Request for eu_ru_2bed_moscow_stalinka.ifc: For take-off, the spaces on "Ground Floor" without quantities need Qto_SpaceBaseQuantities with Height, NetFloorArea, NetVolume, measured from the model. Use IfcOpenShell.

First a look at what the model holds.

```python
import ifcopenshell
import ifcopenshell.util.element
import ifcopenshell.util.unit

model = ifcopenshell.open("eu_ru_2bed_moscow_stalinka.ifc")
print(model.schema)
for unit_type in ("LENGTHUNIT", "AREAUNIT", "VOLUMEUNIT"):
    print(unit_type, ifcopenshell.util.unit.calculate_unit_scale(model, unit_type))
storey = next(s for s in model.by_type("IfcBuildingStorey") if s.Name == "Ground Floor")
spaces = [e for e in ifcopenshell.util.element.get_decomposition(storey) if e.is_a("IfcSpace")]
for e in sorted(spaces, key=lambda e: e.id()):
    print(e.id(), e.is_a(), e.Name, list(ifcopenshell.util.element.get_psets(e, qtos_only=True)), sep=" | ")
```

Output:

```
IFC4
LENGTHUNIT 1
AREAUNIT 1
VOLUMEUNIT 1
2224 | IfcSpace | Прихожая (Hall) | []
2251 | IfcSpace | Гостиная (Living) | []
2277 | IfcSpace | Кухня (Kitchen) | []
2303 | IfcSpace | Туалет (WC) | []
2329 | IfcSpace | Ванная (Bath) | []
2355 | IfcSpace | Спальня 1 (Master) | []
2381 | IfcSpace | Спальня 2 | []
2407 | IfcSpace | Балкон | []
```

```python
import ifcopenshell
import ifcopenshell.api.pset
import ifcopenshell.geom
import ifcopenshell.util.element
import ifcopenshell.util.shape
import ifcopenshell.util.unit

model = ifcopenshell.open("eu_ru_2bed_moscow_stalinka.ifc")
unit_scale = ifcopenshell.util.unit.calculate_unit_scale(model)
area_scale = ifcopenshell.util.unit.calculate_unit_scale(model, "AREAUNIT")
volume_scale = ifcopenshell.util.unit.calculate_unit_scale(model, "VOLUMEUNIT")
settings = ifcopenshell.geom.settings()

storey = next(s for s in model.by_type("IfcBuildingStorey") if s.Name == "Ground Floor")
spaces = [e for e in ifcopenshell.util.element.get_decomposition(storey) if e.is_a("IfcSpace")]

for e in sorted(spaces, key=lambda e: e.id()):
    if ifcopenshell.util.element.get_psets(e, qtos_only=True, should_inherit=False):
        continue
    # Geometry comes back in metres, in the element's own axes.
    shape = ifcopenshell.geom.create_shape(settings, e)
    values = {
        "Height": ifcopenshell.util.shape.get_z(shape.geometry) / unit_scale,
        "NetFloorArea": ifcopenshell.util.shape.get_footprint_area(shape.geometry) / area_scale,
        "NetVolume": ifcopenshell.util.shape.get_volume(shape.geometry) / volume_scale,
    }
    qto = ifcopenshell.api.pset.add_qto(model, product=e, name="Qto_SpaceBaseQuantities")
    ifcopenshell.api.pset.edit_qto(model, qto=qto, properties=values)
    print(e.id(), {k: round(v, 3) for k, v in values.items()})

model.write("eu_ru_2bed_moscow_stalinka_rev.ifc")
```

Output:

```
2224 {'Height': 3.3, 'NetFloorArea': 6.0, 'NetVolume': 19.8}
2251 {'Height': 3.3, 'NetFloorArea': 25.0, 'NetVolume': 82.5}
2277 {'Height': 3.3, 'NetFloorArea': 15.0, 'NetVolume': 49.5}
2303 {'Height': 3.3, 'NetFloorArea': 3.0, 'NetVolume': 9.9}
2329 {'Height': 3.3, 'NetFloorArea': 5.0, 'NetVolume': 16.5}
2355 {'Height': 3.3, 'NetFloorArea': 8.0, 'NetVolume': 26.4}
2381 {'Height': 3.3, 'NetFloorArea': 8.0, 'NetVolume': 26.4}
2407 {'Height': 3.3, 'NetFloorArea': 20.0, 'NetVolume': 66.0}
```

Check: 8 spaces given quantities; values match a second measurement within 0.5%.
